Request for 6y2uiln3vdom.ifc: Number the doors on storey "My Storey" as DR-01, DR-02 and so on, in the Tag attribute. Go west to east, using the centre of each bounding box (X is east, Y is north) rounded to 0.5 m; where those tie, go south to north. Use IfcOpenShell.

First a look at what the model holds.

```python
import ifcopenshell
import ifcopenshell.util.element
import ifcopenshell.util.placement

model = ifcopenshell.open("6y2uiln3vdom.ifc")
print(model.schema)
storey = next(s for s in model.by_type("IfcBuildingStorey") if s.Name == "My Storey")
doors = [e for e in ifcopenshell.util.element.get_decomposition(storey) if e.is_a("IfcDoor")]
for e in sorted(doors, key=lambda e: e.id()):
    origin = ifcopenshell.util.placement.get_local_placement(e.ObjectPlacement)[:3, 3]
    print(e.id(), e.Tag, e.Name, origin.round(2) + 0.0, sep=" | ")
```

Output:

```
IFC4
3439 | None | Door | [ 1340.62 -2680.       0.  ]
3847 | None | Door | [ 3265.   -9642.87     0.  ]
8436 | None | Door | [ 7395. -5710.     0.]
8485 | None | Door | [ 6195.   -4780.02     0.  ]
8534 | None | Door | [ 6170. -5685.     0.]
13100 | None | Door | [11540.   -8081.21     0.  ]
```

```python
import ifcopenshell
import ifcopenshell.geom
import ifcopenshell.util.element
import ifcopenshell.util.shape

model = ifcopenshell.open("6y2uiln3vdom.ifc")
settings = ifcopenshell.geom.settings()
settings.set("use-world-coords", True)


def centre(element):
    shape = ifcopenshell.geom.create_shape(settings, element)
    return ifcopenshell.util.shape.get_bbox_centroid(shape.geometry)


storey = next(s for s in model.by_type("IfcBuildingStorey") if s.Name == "My Storey")
doors = [e for e in ifcopenshell.util.element.get_decomposition(storey) if e.is_a("IfcDoor")]

# Insertion points can sit at a corner or the storey origin, so sort by the geometry (in metres).
centres = {e: centre(e) for e in doors}
doors.sort(key=lambda e: (round(centres[e][0] / 0.5), centres[e][1]))

for i, e in enumerate(doors, start=1):
    number = f"DR-{i:02d}"
    e.Tag = number
    print(e.id(), number)

model.write("6y2uiln3vdom_rev.ifc")
```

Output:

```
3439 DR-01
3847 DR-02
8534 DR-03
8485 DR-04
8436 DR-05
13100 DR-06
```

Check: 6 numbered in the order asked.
